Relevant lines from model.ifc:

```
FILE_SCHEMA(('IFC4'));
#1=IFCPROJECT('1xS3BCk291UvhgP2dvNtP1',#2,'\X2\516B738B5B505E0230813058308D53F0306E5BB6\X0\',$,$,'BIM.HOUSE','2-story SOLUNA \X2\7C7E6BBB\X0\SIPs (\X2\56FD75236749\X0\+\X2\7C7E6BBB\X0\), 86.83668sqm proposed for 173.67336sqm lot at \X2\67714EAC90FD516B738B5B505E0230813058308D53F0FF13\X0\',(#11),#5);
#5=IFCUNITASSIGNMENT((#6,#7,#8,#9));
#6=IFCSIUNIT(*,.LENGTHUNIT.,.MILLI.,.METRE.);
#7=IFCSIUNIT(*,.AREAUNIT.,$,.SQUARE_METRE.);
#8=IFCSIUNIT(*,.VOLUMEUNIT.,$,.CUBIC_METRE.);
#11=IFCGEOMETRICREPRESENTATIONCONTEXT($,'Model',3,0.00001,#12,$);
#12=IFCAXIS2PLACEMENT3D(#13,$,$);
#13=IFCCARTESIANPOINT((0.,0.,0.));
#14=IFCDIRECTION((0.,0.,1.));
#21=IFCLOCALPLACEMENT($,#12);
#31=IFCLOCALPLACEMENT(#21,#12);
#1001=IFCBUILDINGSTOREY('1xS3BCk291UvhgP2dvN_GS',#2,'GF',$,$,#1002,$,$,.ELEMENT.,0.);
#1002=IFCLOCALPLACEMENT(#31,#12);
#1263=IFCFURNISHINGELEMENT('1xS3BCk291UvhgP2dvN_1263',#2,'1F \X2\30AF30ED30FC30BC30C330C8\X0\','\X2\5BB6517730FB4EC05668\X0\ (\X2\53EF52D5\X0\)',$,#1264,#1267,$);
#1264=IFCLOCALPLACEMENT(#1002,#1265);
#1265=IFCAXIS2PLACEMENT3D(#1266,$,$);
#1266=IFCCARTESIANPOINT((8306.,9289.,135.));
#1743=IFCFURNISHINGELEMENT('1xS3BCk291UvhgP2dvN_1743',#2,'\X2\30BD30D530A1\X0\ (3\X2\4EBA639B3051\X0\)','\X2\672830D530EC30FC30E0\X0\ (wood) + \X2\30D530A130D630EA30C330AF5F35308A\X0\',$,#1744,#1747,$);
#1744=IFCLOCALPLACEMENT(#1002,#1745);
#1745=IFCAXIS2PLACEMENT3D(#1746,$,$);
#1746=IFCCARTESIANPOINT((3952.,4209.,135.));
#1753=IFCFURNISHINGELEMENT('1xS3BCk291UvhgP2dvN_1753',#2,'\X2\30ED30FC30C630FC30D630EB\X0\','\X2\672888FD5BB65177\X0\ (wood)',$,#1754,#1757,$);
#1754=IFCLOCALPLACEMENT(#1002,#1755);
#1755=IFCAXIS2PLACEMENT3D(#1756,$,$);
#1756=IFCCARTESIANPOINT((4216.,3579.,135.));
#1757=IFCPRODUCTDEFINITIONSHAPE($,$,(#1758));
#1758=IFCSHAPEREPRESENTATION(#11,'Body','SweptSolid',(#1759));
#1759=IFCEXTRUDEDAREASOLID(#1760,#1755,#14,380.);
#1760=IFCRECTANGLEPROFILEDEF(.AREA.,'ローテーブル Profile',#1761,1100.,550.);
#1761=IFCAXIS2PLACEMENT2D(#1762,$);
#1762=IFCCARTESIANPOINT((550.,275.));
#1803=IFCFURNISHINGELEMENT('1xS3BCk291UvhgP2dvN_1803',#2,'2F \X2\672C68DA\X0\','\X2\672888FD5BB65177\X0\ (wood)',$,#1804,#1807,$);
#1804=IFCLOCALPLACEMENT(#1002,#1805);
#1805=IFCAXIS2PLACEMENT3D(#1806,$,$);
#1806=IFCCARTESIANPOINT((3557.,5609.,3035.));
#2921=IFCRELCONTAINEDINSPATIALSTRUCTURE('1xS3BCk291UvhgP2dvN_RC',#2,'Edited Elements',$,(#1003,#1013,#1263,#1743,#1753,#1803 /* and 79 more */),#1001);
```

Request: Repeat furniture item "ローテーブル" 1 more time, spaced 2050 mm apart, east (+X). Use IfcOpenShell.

```python
import numpy as np
import ifcopenshell
import ifcopenshell.api.geometry
import ifcopenshell.api.root
import ifcopenshell.util.element
import ifcopenshell.util.placement
import ifcopenshell.util.unit

model = ifcopenshell.open("model.ifc")
unit_scale = ifcopenshell.util.unit.calculate_unit_scale(model)


def reuse_history(source, copy):
    """copy_class also copies each property set's owner history, people and application; keep the originals."""
    for rel in copy.IsDefinedBy:
        if rel.is_a("IfcRelDefinesByProperties") and (history := rel.RelatingPropertyDefinition.OwnerHistory):
            rel.RelatingPropertyDefinition.OwnerHistory = source.OwnerHistory
            ifcopenshell.util.element.remove_deep2(model, history)


source = model.by_guid("1xS3BCk291UvhgP2dvN_1753")
base = ifcopenshell.util.placement.get_local_placement(source.ObjectPlacement)
step = np.array([1.0, 0.0, 0.0]) * 2.05 / unit_scale

for i in range(1, 2):
    copy = ifcopenshell.api.root.copy_class(model, product=source)
    copy.Representation = ifcopenshell.util.element.copy_deep(
        model, source.Representation, exclude=["IfcGeometricRepresentationContext", "IfcRepresentationMap"]
    )
    reuse_history(source, copy)
    matrix = base.copy()
    matrix[:3, 3] += i * step
    print("added at", matrix[:3, 3].round(3) + 0.0)
    ifcopenshell.api.geometry.edit_object_placement(model, product=copy, matrix=matrix, is_si=False)

model.write("model_updated.ifc")
```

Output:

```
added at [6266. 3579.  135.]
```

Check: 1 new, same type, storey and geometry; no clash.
